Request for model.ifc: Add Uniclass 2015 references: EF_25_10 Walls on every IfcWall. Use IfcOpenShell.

First a look at what the model holds.

```python
import ifcopenshell

model = ifcopenshell.open("model.ifc")
print(model.schema)
print("classifications:", [c.Name for c in model.by_type("IfcClassification")])
for ifc_class in ("IfcDoor", "IfcRoof", "IfcStair", "IfcWall", "IfcWindow"):
    print(ifc_class, len(model.by_type(ifc_class)))
```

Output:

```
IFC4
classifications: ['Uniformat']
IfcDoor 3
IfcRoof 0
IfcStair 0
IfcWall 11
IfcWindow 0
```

```python
import ifcopenshell
import ifcopenshell.api.classification

model = ifcopenshell.open("model.ifc")

system = ifcopenshell.api.classification.add_classification(model, classification="Uniclass 2015")

codes = {
    "IfcWall": ("EF_25_10", "Walls"),
}
for ifc_class, (code, name) in codes.items():
    products = model.by_type(ifc_class)
    ifcopenshell.api.classification.add_reference(
        model, products=products, classification=system, identification=code, name=name
    )
    print(code, len(products))

model.write("model_updated.ifc")
```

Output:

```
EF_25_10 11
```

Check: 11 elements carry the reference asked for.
